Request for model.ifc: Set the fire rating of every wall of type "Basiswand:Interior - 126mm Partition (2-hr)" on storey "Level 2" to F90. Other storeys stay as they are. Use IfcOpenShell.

First a look at what the model holds.

```python
import ifcopenshell
import ifcopenshell.util.element

model = ifcopenshell.open("model.ifc")
print(model.schema)
storey = next(s for s in model.by_type("IfcBuildingStorey") if s.Name == "Level 2")
walls = [e for e in ifcopenshell.util.element.get_decomposition(storey) if e.is_a("IfcWall")]
seen = {}
for e in walls:
    element_type = ifcopenshell.util.element.get_type(e)
    key = (element_type.Name if element_type != e and element_type else None, ifcopenshell.util.element.get_pset(e, "Pset_WallCommon", "FireRating"))
    seen[key] = seen.get(key, 0) + 1
for (name, value), count in sorted(seen.items(), key=str):
    print(count, "x", name, "|", value)
```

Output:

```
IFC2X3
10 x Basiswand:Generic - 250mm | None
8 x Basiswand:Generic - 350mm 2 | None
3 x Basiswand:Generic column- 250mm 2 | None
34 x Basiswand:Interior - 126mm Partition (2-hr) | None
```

```python
import ifcopenshell
import ifcopenshell.api.pset
import ifcopenshell.util.element

model = ifcopenshell.open("model.ifc")

storey = next(s for s in model.by_type("IfcBuildingStorey") if s.Name == "Level 2")
walls = [e for e in ifcopenshell.util.element.get_decomposition(storey) if e.is_a("IfcWall")]

count = 0
for e in walls:
    element_type = ifcopenshell.util.element.get_type(e)
    if element_type in (None, e) or element_type.Name != "Basiswand:Interior - 126mm Partition (2-hr)":
        continue
    # add_pset returns the element's existing set when there is one.
    pset = ifcopenshell.api.pset.add_pset(model, product=e, name="Pset_WallCommon")
    ifcopenshell.api.pset.edit_pset(model, pset=pset, properties={"FireRating": "F90"})
    count += 1

print(count, "walls updated")

model.write("model_rev.ifc")
```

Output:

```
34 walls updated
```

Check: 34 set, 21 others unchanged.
